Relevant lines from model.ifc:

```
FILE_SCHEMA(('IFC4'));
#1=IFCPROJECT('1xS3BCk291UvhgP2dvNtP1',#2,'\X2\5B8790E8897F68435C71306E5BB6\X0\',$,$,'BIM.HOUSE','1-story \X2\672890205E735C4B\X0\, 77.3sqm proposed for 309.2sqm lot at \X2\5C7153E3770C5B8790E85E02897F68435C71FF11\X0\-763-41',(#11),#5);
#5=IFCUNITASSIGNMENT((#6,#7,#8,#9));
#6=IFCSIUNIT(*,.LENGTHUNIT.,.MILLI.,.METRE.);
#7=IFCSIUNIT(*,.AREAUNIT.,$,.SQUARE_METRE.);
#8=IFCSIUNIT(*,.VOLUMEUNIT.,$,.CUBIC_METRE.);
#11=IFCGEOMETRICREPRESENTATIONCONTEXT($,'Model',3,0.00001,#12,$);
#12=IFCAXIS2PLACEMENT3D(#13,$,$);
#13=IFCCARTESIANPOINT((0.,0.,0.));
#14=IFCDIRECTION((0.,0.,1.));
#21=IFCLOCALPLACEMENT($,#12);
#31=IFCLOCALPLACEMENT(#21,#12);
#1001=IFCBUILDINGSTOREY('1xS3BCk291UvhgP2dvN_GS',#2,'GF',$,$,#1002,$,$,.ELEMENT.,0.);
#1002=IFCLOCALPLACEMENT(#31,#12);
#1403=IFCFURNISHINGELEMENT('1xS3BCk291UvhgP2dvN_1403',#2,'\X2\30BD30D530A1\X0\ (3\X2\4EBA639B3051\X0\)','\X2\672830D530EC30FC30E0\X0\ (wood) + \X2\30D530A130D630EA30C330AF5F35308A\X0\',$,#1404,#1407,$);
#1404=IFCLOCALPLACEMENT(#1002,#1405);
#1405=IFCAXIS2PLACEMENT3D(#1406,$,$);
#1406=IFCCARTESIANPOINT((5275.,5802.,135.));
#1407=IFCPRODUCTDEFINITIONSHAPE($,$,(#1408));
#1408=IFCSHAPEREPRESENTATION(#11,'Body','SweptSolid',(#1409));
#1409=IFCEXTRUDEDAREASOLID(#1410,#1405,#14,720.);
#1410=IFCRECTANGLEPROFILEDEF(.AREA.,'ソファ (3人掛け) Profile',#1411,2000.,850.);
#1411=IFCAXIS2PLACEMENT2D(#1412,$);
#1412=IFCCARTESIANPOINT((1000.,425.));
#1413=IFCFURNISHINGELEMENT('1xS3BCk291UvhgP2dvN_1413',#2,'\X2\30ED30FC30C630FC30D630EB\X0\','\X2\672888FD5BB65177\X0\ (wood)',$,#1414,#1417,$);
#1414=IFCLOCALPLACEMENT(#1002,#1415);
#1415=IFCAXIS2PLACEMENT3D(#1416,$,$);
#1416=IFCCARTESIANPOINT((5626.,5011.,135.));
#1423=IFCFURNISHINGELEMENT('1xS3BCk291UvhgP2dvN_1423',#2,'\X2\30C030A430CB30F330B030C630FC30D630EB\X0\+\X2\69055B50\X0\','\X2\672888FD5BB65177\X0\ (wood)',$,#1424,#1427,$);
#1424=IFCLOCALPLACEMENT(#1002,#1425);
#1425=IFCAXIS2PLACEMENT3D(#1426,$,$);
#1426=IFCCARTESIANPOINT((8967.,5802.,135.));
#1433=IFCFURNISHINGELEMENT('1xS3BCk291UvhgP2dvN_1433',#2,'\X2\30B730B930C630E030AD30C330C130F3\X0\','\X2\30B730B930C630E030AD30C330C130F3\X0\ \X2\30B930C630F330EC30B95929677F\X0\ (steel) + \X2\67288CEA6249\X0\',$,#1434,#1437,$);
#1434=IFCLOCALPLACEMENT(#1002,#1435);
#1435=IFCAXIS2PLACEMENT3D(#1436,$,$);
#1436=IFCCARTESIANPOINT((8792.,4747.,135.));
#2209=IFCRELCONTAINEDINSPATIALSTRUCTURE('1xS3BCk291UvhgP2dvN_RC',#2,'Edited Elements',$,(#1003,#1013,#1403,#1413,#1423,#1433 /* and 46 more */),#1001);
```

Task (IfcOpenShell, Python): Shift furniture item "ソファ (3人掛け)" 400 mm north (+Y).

```python
import ifcopenshell
import ifcopenshell.api.geometry
import ifcopenshell.util.placement

model = ifcopenshell.open("model.ifc")

item = model.by_guid("1xS3BCk291UvhgP2dvN_1403")
matrix = ifcopenshell.util.placement.get_local_placement(item.ObjectPlacement)
matrix[1, 3] += 400.0
ifcopenshell.api.geometry.edit_object_placement(model, product=item, matrix=matrix, is_si=False)

print(ifcopenshell.util.placement.get_local_placement(item.ObjectPlacement).round(3) + 0.0)

model.write("model-out.ifc")
```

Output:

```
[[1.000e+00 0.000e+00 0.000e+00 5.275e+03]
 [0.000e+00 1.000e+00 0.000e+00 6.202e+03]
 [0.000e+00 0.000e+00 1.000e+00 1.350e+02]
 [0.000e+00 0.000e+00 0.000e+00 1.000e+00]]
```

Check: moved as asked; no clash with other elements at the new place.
